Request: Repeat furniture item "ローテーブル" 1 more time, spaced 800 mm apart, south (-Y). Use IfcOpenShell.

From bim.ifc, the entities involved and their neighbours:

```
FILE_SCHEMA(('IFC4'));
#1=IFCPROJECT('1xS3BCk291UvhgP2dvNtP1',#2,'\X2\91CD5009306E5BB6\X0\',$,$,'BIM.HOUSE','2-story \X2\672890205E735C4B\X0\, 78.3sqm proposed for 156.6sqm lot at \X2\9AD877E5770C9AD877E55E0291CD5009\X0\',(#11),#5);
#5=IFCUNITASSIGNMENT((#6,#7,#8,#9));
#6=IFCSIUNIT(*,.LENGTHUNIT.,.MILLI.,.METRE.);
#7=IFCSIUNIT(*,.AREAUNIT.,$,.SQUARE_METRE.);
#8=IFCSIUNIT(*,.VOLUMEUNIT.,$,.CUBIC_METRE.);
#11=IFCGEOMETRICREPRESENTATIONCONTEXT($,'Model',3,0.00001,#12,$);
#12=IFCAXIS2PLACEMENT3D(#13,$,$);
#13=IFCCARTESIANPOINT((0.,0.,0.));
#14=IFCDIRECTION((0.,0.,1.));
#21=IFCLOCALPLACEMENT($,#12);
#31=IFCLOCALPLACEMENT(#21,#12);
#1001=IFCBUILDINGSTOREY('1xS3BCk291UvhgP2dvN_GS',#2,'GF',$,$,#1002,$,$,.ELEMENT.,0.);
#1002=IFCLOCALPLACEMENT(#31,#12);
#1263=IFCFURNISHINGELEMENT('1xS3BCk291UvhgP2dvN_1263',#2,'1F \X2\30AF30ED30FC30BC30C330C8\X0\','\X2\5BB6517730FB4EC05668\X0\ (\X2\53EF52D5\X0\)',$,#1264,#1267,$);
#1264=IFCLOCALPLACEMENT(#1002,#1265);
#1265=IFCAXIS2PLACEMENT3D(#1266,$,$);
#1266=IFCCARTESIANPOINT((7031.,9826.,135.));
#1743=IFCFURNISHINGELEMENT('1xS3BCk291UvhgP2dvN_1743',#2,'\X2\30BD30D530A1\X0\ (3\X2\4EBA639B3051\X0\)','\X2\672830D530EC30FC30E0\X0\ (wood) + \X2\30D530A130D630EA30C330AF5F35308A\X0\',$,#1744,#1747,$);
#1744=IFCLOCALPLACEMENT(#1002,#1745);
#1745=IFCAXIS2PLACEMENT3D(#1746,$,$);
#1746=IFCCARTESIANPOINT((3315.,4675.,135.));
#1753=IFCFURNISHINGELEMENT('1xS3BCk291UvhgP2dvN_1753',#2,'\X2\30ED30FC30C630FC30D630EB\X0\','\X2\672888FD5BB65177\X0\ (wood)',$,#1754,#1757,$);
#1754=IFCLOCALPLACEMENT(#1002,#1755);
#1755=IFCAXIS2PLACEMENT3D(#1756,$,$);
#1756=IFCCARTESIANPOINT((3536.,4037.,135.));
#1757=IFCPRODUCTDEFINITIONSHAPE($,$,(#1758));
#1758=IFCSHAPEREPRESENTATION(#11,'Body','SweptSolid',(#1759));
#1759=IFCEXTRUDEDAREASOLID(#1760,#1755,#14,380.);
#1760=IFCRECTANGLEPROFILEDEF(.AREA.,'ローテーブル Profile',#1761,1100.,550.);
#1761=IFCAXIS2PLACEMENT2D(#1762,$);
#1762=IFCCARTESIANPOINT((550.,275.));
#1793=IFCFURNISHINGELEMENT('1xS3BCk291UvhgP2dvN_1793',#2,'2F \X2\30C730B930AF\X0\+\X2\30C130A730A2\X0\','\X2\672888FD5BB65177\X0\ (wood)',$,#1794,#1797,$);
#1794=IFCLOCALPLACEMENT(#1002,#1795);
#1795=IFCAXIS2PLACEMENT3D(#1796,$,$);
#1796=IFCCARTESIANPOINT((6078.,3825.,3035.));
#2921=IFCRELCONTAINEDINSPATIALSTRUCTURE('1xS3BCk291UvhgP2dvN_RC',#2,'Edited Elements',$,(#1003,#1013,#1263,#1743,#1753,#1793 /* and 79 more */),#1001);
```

```python
import numpy as np
import ifcopenshell
import ifcopenshell.api.geometry
import ifcopenshell.api.root
import ifcopenshell.util.element
import ifcopenshell.util.placement
import ifcopenshell.util.unit

model = ifcopenshell.open("bim.ifc")
unit_scale = ifcopenshell.util.unit.calculate_unit_scale(model)


def reuse_history(source, copy):
    """copy_class also copies each property set's owner history, people and application; keep the originals."""
    for rel in copy.IsDefinedBy:
        if rel.is_a("IfcRelDefinesByProperties") and (history := rel.RelatingPropertyDefinition.OwnerHistory):
            rel.RelatingPropertyDefinition.OwnerHistory = source.OwnerHistory
            ifcopenshell.util.element.remove_deep2(model, history)


source = model.by_guid("1xS3BCk291UvhgP2dvN_1753")
base = ifcopenshell.util.placement.get_local_placement(source.ObjectPlacement)
step = np.array([0.0, -1.0, 0.0]) * 0.8 / unit_scale

for i in range(1, 2):
    copy = ifcopenshell.api.root.copy_class(model, product=source)
    copy.Representation = ifcopenshell.util.element.copy_deep(
        model, source.Representation, exclude=["IfcGeometricRepresentationContext", "IfcRepresentationMap"]
    )
    reuse_history(source, copy)
    matrix = base.copy()
    matrix[:3, 3] += i * step
    print("added at", matrix[:3, 3].round(3) + 0.0)
    ifcopenshell.api.geometry.edit_object_placement(model, product=copy, matrix=matrix, is_si=False)

model.write("bim_updated.ifc")
```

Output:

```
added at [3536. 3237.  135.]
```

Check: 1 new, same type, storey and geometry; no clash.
